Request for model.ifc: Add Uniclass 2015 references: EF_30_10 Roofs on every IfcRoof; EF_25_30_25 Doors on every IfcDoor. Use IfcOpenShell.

First a look at what the model holds.

```python
import ifcopenshell

model = ifcopenshell.open("model.ifc")
print(model.schema)
print("classifications:", [c.Name for c in model.by_type("IfcClassification")])
for ifc_class in ("IfcDoor", "IfcRoof", "IfcStair", "IfcWall", "IfcWindow"):
    print(ifc_class, len(model.by_type(ifc_class)))
```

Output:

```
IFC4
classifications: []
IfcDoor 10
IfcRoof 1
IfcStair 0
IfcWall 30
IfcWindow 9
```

```python
import ifcopenshell
import ifcopenshell.api.classification

model = ifcopenshell.open("model.ifc")

system = ifcopenshell.api.classification.add_classification(model, classification="Uniclass 2015")

codes = {
    "IfcRoof": ("EF_30_10", "Roofs"),
    "IfcDoor": ("EF_25_30_25", "Doors"),
}
for ifc_class, (code, name) in codes.items():
    products = model.by_type(ifc_class)
    ifcopenshell.api.classification.add_reference(
        model, products=products, classification=system, identification=code, name=name
    )
    print(code, len(products))

model.write("model_updated.ifc")
```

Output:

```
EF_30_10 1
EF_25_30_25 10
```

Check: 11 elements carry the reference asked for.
